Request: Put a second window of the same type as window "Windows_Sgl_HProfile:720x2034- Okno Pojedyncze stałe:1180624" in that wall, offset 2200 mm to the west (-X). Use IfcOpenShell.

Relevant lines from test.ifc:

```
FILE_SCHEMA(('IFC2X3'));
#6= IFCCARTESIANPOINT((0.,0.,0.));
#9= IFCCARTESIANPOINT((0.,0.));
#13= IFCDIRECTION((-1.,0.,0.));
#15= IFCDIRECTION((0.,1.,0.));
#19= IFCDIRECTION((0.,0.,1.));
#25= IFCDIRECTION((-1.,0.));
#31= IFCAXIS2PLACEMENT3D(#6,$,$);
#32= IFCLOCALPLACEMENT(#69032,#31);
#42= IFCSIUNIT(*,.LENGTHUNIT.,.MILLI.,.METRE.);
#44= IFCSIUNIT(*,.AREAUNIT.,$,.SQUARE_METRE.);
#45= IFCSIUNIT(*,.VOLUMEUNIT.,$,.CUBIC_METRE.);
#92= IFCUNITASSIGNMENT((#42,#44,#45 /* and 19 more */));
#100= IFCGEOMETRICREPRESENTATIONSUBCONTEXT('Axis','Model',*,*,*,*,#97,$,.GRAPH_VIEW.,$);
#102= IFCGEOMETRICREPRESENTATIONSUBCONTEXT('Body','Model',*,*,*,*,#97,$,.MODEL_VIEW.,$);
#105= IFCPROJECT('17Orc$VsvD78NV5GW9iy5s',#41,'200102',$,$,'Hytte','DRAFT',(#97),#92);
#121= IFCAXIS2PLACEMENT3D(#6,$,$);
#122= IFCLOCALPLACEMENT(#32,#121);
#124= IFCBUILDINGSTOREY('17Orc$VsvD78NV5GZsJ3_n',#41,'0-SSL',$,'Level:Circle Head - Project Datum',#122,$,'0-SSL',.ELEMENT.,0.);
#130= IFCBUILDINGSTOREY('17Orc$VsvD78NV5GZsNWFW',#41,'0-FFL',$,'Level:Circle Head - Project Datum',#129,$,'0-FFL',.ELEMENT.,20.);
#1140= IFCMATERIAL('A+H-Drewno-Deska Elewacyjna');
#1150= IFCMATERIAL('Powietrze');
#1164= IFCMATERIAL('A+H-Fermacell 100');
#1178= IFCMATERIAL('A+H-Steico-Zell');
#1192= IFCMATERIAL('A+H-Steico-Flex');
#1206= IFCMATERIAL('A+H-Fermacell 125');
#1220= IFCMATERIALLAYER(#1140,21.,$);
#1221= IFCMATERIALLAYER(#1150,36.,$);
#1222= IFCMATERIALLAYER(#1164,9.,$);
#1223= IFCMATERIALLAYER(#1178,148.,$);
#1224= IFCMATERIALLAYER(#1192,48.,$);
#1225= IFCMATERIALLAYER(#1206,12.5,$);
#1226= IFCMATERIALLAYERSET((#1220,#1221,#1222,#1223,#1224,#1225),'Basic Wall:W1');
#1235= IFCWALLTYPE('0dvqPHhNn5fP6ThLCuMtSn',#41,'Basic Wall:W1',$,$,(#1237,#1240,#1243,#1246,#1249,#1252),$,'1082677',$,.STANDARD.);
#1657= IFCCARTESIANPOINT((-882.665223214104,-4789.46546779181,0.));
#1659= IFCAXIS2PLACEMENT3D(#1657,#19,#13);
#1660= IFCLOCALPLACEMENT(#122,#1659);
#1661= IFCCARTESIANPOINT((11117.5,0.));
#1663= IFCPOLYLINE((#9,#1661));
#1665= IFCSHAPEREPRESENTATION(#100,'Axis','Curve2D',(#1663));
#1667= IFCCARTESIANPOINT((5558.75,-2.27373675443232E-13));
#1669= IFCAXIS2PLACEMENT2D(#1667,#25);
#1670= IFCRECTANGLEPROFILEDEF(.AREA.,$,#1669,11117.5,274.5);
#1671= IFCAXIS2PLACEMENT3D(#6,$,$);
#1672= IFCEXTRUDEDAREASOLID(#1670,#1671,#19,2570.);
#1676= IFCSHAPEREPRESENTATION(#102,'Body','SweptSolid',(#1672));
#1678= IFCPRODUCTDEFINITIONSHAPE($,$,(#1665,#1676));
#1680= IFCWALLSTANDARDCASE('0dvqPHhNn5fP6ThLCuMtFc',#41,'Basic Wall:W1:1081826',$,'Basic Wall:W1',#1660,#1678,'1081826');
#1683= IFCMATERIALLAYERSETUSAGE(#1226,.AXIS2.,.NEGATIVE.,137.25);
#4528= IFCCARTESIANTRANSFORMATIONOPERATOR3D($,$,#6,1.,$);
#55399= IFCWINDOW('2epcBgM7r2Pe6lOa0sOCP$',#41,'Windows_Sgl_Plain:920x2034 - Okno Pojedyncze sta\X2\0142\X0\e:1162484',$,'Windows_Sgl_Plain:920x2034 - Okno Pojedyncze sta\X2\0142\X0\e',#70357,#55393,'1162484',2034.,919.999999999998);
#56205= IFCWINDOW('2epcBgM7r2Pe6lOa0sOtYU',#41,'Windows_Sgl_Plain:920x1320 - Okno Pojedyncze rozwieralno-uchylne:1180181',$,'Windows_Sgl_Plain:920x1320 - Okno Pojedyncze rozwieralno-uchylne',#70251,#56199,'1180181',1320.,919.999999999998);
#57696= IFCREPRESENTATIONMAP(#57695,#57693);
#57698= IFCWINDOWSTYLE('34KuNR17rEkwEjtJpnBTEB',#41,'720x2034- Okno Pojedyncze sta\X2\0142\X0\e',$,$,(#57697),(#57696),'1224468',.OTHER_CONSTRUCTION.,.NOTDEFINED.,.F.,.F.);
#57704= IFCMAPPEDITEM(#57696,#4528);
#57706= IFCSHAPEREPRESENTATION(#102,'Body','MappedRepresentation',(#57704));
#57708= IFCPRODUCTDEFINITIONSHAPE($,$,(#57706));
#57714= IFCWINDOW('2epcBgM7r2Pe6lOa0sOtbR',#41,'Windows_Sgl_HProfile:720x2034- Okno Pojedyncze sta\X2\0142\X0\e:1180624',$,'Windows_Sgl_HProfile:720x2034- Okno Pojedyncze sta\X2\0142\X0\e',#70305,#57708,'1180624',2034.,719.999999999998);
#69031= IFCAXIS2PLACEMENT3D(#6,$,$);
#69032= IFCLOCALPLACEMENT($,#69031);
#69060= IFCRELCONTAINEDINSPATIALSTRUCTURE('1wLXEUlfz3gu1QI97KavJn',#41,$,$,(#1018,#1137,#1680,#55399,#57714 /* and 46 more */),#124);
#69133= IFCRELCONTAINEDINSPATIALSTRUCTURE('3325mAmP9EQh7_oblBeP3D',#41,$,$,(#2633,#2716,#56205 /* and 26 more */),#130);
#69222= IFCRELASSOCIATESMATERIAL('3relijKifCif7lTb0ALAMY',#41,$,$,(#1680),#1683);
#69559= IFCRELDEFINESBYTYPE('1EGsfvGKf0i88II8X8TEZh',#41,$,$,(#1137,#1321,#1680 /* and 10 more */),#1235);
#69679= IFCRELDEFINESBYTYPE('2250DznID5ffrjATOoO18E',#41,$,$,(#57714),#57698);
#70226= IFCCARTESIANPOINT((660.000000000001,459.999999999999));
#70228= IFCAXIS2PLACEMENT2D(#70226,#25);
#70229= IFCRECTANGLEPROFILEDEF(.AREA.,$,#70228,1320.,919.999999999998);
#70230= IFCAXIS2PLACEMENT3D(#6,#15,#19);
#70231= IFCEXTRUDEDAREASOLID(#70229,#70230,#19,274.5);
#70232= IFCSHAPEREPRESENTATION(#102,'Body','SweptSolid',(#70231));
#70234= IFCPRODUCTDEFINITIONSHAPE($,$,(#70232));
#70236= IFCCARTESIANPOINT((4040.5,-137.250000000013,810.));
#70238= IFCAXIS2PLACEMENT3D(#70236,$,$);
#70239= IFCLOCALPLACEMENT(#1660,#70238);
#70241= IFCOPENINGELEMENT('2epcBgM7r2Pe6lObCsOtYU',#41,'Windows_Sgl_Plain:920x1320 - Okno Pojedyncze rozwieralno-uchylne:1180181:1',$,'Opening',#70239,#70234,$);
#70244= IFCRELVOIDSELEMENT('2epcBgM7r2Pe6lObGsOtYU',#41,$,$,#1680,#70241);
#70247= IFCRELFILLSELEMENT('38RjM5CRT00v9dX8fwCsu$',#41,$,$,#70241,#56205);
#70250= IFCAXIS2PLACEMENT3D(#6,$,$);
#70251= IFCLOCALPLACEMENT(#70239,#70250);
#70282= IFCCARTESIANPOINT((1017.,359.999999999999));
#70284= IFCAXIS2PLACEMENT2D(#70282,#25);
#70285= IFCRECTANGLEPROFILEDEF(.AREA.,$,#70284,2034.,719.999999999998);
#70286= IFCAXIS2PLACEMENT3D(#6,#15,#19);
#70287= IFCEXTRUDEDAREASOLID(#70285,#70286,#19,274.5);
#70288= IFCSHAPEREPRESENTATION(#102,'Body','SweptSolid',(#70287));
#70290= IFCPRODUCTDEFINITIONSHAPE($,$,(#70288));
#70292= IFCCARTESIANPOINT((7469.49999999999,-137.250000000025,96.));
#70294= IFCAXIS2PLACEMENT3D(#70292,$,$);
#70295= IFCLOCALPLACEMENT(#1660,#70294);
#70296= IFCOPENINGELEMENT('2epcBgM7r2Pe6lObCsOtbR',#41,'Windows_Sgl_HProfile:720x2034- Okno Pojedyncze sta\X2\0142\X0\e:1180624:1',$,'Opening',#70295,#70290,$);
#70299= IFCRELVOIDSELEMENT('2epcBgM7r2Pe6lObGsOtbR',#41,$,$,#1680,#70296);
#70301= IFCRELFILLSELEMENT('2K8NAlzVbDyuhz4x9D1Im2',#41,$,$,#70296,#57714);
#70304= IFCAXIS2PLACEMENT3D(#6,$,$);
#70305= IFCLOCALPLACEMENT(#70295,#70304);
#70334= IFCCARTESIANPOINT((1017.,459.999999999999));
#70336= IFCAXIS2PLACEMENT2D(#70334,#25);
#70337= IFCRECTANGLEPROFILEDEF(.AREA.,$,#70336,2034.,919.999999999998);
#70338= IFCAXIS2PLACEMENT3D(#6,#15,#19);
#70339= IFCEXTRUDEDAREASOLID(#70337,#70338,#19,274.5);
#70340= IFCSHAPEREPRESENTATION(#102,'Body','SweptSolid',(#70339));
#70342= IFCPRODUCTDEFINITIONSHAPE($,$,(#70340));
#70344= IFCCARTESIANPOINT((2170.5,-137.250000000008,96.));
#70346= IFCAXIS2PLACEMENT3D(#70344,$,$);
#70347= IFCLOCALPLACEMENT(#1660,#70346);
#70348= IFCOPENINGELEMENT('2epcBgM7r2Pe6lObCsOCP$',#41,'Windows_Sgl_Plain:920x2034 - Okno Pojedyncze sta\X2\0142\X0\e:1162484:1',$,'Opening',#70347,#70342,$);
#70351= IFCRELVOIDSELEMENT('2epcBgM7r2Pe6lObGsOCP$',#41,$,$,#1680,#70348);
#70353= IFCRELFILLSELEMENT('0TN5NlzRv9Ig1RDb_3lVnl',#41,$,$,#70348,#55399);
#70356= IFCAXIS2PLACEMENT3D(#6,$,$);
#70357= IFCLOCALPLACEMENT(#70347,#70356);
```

```python
import ifcopenshell
import ifcopenshell.api.feature
import ifcopenshell.api.geometry
import ifcopenshell.api.root
import ifcopenshell.geom
import ifcopenshell.util.element
import ifcopenshell.util.placement
import ifcopenshell.util.shape
import ifcopenshell.util.unit

model = ifcopenshell.open("test.ifc")
unit_scale = ifcopenshell.util.unit.calculate_unit_scale(model)
settings = ifcopenshell.geom.settings()


def volume(element):
    """Net volume in cubic metres, openings subtracted."""
    shape = ifcopenshell.geom.create_shape(settings, element)
    return ifcopenshell.util.shape.get_volume(shape.geometry)


def reuse_history(source, copy):
    """copy_class also copies each property set's owner history, people and application; keep the originals."""
    for rel in copy.IsDefinedBy:
        if rel.is_a("IfcRelDefinesByProperties") and (history := rel.RelatingPropertyDefinition.OwnerHistory):
            rel.RelatingPropertyDefinition.OwnerHistory = source.OwnerHistory
            ifcopenshell.util.element.remove_deep2(model, history)


window = model.by_guid("2epcBgM7r2Pe6lOa0sOtbR")
opening = window.FillsVoids[0].RelatingOpeningElement
wall = opening.VoidsElements[0].RelatingBuildingElement
before = volume(wall)
shift = ifcopenshell.util.placement.get_local_placement(wall.ObjectPlacement)[:3, 0] * 2.2 / unit_scale

# copy_class copies the void relationship, type, container and properties, but no geometry.
new_opening = ifcopenshell.api.root.copy_class(model, product=opening)
new_opening.Representation = ifcopenshell.util.element.copy_deep(
    model, opening.Representation, exclude=["IfcGeometricRepresentationContext", "IfcRepresentationMap"]
)
new_opening.Name = "Windows_Sgl_HProfile:720x2034- Okno Pojedyncze stałe"
new_window = ifcopenshell.api.root.copy_class(model, product=window)
new_window.Representation = ifcopenshell.util.element.copy_deep(
    model, window.Representation, exclude=["IfcGeometricRepresentationContext", "IfcRepresentationMap"]
)
new_window.Name = "Windows_Sgl_HProfile:720x2034- Okno Pojedyncze stałe"
new_window.Tag = None
reuse_history(window, new_window)
fills = ifcopenshell.api.feature.add_filling(model, opening=new_opening, element=new_window)
fills.OwnerHistory = new_window.OwnerHistory  # required in IFC2X3

for old, new in ((opening, new_opening), (window, new_window)):
    matrix = ifcopenshell.util.placement.get_local_placement(old.ObjectPlacement)
    matrix[:3, 3] += shift
    ifcopenshell.api.geometry.edit_object_placement(model, product=new, matrix=matrix, is_si=False)

after = volume(wall)

print(f"wall volume {before:.3f} -> {after:.3f} m3")

model.write("test_updated.ifc")
```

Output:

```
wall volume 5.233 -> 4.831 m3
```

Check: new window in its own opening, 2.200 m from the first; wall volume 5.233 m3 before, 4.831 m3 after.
